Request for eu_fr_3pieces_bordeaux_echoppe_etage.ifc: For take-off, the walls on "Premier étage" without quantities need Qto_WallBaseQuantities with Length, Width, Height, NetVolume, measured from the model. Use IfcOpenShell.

First a look at what the model holds.

```python
import ifcopenshell
import ifcopenshell.util.element
import ifcopenshell.util.unit

model = ifcopenshell.open("eu_fr_3pieces_bordeaux_echoppe_etage.ifc")
print(model.schema)
for unit_type in ("LENGTHUNIT", "AREAUNIT", "VOLUMEUNIT"):
    print(unit_type, ifcopenshell.util.unit.calculate_unit_scale(model, unit_type))
storey = next(s for s in model.by_type("IfcBuildingStorey") if s.Name == "Premier étage")
walls = [e for e in ifcopenshell.util.element.get_decomposition(storey) if e.is_a("IfcWall")]
for e in sorted(walls, key=lambda e: e.id()):
    print(e.id(), e.is_a(), e.Name, list(ifcopenshell.util.element.get_psets(e, qtos_only=True)), sep=" | ")
```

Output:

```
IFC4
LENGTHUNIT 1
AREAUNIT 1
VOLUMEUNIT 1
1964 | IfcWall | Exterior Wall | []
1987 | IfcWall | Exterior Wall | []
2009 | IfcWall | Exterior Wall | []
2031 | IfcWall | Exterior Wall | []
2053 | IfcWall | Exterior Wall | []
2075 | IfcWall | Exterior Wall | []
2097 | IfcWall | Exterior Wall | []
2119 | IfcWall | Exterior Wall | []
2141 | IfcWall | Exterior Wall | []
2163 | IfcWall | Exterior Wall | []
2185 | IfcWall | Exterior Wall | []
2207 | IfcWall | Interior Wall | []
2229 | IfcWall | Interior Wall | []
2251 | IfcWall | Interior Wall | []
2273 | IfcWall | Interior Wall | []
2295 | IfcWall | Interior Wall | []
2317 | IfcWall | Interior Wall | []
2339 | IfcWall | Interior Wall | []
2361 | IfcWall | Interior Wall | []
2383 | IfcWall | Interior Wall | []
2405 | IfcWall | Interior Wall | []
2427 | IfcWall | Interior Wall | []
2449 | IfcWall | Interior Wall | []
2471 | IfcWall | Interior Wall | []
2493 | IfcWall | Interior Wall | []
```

```python
import ifcopenshell
import ifcopenshell.api.pset
import ifcopenshell.geom
import ifcopenshell.util.element
import ifcopenshell.util.shape
import ifcopenshell.util.unit

model = ifcopenshell.open("eu_fr_3pieces_bordeaux_echoppe_etage.ifc")
unit_scale = ifcopenshell.util.unit.calculate_unit_scale(model)
volume_scale = ifcopenshell.util.unit.calculate_unit_scale(model, "VOLUMEUNIT")
settings = ifcopenshell.geom.settings()

storey = next(s for s in model.by_type("IfcBuildingStorey") if s.Name == "Premier étage")
walls = [e for e in ifcopenshell.util.element.get_decomposition(storey) if e.is_a("IfcWall")]

for e in sorted(walls, key=lambda e: e.id()):
    if ifcopenshell.util.element.get_psets(e, qtos_only=True, should_inherit=False):
        continue
    # Geometry comes back in metres, in the element's own axes.
    shape = ifcopenshell.geom.create_shape(settings, e)
    values = {
        "Length": ifcopenshell.util.shape.get_x(shape.geometry) / unit_scale,
        "Width": ifcopenshell.util.shape.get_y(shape.geometry) / unit_scale,
        "Height": ifcopenshell.util.shape.get_z(shape.geometry) / unit_scale,
        "NetVolume": ifcopenshell.util.shape.get_volume(shape.geometry) / volume_scale,
    }
    qto = ifcopenshell.api.pset.add_qto(model, product=e, name="Qto_WallBaseQuantities")
    ifcopenshell.api.pset.edit_qto(model, qto=qto, properties=values)
    print(e.id(), {k: round(v, 3) for k, v in values.items()})

model.write("eu_fr_3pieces_bordeaux_echoppe_etage_edited.ifc")
```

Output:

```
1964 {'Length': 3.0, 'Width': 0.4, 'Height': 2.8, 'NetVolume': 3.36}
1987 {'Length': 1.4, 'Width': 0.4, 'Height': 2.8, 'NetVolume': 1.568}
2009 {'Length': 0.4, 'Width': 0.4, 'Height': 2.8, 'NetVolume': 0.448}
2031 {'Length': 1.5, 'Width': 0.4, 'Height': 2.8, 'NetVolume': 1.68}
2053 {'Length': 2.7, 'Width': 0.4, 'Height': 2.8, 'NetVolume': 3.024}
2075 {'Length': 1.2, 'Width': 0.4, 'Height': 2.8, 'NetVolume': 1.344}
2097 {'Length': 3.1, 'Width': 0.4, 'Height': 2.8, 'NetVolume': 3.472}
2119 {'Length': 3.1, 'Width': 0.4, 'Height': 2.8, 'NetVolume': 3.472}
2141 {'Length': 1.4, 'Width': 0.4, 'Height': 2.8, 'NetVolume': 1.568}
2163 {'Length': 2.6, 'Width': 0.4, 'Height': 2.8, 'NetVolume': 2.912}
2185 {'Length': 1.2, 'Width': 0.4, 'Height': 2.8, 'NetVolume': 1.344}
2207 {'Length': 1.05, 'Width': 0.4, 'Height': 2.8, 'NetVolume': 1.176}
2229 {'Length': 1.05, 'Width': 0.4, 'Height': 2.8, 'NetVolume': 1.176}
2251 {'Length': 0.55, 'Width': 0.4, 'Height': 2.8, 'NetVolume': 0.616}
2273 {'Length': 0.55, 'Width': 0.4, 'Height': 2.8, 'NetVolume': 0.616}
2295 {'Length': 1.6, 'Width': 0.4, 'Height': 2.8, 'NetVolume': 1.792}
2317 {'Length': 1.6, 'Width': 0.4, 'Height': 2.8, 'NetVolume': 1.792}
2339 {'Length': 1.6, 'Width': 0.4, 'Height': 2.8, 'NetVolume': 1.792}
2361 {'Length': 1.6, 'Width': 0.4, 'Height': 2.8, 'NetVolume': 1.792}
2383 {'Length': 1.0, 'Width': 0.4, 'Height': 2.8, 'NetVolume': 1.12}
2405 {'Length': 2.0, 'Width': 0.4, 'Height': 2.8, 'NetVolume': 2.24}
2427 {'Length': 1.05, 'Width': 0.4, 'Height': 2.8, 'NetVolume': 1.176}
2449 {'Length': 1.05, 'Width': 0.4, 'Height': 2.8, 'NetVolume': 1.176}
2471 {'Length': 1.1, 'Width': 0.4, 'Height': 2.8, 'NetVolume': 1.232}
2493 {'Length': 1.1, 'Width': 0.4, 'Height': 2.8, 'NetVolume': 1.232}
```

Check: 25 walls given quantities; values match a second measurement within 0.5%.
